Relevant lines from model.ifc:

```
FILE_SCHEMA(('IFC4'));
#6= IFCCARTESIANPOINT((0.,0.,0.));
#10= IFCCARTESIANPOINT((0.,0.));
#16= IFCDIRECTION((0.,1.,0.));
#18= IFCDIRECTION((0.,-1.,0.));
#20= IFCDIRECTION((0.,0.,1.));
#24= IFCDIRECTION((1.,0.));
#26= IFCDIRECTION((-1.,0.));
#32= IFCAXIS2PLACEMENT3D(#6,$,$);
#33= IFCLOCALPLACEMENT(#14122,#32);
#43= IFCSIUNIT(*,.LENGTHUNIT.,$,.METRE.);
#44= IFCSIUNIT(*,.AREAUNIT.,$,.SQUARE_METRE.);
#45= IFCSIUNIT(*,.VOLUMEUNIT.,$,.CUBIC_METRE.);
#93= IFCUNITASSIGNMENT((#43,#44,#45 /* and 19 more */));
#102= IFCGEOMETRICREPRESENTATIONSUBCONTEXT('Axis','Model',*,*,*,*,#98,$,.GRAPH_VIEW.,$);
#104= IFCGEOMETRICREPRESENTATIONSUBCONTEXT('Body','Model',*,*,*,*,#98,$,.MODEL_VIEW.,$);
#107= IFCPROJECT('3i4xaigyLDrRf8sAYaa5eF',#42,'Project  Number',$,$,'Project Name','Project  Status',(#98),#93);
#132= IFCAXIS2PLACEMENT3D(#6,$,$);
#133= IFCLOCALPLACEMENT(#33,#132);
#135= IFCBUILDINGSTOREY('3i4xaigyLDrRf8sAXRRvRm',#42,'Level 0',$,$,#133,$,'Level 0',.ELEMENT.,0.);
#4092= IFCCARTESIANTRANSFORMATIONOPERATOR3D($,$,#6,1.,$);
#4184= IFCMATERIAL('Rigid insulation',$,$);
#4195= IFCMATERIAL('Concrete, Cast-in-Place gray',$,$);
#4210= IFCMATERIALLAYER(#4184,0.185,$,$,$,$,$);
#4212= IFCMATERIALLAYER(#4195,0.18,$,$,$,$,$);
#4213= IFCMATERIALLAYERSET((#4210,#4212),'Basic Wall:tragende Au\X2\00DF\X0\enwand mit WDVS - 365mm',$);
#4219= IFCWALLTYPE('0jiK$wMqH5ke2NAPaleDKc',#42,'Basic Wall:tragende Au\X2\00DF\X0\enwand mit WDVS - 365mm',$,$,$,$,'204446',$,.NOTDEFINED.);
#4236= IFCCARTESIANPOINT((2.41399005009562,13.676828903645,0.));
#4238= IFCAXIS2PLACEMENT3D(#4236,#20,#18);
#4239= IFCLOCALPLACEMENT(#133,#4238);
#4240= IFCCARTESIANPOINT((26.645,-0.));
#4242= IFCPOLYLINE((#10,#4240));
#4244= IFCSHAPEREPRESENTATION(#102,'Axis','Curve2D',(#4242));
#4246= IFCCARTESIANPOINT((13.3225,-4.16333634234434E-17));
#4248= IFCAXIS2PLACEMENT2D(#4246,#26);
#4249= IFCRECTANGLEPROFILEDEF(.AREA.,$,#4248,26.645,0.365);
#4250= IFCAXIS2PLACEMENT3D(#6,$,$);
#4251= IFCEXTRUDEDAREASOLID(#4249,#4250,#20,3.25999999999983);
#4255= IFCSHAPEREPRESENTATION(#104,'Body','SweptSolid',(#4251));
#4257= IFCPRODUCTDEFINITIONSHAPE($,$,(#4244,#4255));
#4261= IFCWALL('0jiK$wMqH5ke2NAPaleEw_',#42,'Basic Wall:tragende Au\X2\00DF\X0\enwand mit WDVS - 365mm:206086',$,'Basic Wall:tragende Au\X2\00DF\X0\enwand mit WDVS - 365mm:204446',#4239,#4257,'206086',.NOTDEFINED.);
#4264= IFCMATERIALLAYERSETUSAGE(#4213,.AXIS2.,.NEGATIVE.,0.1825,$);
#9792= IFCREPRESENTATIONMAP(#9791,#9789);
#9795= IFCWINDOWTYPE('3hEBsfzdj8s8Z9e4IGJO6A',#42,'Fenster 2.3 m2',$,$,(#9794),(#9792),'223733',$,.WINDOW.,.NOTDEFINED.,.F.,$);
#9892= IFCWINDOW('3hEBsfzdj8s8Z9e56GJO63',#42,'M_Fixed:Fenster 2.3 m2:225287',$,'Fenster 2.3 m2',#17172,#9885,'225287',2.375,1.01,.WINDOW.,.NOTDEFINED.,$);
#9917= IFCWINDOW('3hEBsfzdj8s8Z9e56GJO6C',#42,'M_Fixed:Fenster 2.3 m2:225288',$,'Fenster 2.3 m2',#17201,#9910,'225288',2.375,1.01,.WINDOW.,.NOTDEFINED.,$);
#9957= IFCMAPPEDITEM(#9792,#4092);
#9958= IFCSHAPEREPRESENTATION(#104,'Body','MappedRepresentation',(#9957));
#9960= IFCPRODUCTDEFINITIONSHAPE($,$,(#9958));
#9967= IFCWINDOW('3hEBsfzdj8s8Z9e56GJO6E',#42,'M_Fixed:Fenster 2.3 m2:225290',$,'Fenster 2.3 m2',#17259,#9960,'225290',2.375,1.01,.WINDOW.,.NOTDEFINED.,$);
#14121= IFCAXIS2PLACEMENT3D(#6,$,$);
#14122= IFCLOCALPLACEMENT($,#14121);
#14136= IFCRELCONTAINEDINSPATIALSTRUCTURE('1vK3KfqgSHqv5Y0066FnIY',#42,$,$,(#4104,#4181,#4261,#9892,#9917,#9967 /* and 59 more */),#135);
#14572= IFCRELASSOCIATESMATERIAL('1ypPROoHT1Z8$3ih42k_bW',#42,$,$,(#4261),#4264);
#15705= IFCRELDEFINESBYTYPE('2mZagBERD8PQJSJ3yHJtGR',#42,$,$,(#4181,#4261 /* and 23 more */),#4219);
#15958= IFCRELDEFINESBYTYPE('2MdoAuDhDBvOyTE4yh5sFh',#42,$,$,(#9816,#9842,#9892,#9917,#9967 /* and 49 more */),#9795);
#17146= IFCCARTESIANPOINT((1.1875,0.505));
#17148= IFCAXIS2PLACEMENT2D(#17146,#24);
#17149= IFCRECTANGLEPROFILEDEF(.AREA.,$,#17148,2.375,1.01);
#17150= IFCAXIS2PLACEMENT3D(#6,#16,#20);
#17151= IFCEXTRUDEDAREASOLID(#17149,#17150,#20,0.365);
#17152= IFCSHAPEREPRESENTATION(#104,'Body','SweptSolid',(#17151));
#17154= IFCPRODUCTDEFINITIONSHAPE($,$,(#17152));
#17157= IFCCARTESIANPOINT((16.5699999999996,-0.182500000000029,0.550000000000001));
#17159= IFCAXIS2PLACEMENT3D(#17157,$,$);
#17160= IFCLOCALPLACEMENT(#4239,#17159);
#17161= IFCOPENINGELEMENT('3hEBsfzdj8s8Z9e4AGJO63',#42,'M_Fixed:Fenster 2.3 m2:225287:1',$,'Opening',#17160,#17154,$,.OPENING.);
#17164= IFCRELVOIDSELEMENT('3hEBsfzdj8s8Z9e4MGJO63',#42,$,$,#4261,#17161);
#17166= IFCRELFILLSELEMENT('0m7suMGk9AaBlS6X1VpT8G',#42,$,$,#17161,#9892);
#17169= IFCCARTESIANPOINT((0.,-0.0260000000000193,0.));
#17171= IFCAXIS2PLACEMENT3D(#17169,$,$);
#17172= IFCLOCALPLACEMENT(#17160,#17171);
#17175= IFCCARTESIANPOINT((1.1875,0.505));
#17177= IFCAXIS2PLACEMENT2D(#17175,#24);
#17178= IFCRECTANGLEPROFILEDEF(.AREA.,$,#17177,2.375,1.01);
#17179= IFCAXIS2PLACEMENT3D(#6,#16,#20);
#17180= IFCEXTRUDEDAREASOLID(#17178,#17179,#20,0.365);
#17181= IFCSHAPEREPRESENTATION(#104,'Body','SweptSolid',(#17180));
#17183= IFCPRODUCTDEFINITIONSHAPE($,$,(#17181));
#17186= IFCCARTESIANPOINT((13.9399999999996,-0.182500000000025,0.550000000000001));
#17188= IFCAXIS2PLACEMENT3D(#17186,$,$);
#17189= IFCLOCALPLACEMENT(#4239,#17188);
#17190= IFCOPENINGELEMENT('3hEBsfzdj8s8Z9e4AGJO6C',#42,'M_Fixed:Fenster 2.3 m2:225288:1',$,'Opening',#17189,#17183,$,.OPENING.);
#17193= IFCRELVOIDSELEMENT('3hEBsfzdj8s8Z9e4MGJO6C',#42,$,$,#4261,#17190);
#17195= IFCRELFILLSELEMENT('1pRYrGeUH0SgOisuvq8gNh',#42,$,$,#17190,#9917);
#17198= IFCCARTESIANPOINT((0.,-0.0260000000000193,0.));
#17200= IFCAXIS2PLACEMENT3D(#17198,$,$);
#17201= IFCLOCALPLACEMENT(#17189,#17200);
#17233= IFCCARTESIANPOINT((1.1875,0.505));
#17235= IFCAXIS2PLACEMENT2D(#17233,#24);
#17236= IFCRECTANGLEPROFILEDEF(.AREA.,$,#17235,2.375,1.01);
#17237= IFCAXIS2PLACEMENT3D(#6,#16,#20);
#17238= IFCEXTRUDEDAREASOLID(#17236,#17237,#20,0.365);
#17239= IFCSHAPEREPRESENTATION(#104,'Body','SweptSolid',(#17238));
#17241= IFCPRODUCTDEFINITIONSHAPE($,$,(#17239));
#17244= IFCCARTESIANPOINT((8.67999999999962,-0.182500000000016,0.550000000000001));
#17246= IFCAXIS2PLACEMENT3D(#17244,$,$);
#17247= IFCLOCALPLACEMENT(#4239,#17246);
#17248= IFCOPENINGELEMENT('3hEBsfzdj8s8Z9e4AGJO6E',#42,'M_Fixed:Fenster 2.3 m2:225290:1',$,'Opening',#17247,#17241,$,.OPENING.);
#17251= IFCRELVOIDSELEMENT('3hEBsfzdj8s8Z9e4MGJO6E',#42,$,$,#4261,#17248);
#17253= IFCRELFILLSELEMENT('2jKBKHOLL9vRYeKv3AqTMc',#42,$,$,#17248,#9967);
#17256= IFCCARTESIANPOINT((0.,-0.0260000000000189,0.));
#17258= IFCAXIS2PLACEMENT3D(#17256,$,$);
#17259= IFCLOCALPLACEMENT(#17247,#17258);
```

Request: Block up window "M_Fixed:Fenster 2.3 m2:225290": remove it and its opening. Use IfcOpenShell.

```python
import ifcopenshell
import ifcopenshell.api.feature
import ifcopenshell.api.root
import ifcopenshell.geom
import ifcopenshell.util.shape

model = ifcopenshell.open("model.ifc")
settings = ifcopenshell.geom.settings()


def volume(element):
    """Net volume in cubic metres, openings subtracted."""
    shape = ifcopenshell.geom.create_shape(settings, element)
    return ifcopenshell.util.shape.get_volume(shape.geometry)


window = model.by_guid("3hEBsfzdj8s8Z9e56GJO6E")
opening = window.FillsVoids[0].RelatingOpeningElement
wall = opening.VoidsElements[0].RelatingBuildingElement
before = volume(wall)

ifcopenshell.api.root.remove_product(model, product=window)
ifcopenshell.api.feature.remove_feature(model, feature=opening)

after = volume(wall)

print(f"wall volume {before:.3f} -> {after:.3f} m3")

model.write("model_updated.ifc")
```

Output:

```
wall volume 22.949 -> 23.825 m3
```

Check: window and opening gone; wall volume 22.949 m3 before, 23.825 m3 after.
